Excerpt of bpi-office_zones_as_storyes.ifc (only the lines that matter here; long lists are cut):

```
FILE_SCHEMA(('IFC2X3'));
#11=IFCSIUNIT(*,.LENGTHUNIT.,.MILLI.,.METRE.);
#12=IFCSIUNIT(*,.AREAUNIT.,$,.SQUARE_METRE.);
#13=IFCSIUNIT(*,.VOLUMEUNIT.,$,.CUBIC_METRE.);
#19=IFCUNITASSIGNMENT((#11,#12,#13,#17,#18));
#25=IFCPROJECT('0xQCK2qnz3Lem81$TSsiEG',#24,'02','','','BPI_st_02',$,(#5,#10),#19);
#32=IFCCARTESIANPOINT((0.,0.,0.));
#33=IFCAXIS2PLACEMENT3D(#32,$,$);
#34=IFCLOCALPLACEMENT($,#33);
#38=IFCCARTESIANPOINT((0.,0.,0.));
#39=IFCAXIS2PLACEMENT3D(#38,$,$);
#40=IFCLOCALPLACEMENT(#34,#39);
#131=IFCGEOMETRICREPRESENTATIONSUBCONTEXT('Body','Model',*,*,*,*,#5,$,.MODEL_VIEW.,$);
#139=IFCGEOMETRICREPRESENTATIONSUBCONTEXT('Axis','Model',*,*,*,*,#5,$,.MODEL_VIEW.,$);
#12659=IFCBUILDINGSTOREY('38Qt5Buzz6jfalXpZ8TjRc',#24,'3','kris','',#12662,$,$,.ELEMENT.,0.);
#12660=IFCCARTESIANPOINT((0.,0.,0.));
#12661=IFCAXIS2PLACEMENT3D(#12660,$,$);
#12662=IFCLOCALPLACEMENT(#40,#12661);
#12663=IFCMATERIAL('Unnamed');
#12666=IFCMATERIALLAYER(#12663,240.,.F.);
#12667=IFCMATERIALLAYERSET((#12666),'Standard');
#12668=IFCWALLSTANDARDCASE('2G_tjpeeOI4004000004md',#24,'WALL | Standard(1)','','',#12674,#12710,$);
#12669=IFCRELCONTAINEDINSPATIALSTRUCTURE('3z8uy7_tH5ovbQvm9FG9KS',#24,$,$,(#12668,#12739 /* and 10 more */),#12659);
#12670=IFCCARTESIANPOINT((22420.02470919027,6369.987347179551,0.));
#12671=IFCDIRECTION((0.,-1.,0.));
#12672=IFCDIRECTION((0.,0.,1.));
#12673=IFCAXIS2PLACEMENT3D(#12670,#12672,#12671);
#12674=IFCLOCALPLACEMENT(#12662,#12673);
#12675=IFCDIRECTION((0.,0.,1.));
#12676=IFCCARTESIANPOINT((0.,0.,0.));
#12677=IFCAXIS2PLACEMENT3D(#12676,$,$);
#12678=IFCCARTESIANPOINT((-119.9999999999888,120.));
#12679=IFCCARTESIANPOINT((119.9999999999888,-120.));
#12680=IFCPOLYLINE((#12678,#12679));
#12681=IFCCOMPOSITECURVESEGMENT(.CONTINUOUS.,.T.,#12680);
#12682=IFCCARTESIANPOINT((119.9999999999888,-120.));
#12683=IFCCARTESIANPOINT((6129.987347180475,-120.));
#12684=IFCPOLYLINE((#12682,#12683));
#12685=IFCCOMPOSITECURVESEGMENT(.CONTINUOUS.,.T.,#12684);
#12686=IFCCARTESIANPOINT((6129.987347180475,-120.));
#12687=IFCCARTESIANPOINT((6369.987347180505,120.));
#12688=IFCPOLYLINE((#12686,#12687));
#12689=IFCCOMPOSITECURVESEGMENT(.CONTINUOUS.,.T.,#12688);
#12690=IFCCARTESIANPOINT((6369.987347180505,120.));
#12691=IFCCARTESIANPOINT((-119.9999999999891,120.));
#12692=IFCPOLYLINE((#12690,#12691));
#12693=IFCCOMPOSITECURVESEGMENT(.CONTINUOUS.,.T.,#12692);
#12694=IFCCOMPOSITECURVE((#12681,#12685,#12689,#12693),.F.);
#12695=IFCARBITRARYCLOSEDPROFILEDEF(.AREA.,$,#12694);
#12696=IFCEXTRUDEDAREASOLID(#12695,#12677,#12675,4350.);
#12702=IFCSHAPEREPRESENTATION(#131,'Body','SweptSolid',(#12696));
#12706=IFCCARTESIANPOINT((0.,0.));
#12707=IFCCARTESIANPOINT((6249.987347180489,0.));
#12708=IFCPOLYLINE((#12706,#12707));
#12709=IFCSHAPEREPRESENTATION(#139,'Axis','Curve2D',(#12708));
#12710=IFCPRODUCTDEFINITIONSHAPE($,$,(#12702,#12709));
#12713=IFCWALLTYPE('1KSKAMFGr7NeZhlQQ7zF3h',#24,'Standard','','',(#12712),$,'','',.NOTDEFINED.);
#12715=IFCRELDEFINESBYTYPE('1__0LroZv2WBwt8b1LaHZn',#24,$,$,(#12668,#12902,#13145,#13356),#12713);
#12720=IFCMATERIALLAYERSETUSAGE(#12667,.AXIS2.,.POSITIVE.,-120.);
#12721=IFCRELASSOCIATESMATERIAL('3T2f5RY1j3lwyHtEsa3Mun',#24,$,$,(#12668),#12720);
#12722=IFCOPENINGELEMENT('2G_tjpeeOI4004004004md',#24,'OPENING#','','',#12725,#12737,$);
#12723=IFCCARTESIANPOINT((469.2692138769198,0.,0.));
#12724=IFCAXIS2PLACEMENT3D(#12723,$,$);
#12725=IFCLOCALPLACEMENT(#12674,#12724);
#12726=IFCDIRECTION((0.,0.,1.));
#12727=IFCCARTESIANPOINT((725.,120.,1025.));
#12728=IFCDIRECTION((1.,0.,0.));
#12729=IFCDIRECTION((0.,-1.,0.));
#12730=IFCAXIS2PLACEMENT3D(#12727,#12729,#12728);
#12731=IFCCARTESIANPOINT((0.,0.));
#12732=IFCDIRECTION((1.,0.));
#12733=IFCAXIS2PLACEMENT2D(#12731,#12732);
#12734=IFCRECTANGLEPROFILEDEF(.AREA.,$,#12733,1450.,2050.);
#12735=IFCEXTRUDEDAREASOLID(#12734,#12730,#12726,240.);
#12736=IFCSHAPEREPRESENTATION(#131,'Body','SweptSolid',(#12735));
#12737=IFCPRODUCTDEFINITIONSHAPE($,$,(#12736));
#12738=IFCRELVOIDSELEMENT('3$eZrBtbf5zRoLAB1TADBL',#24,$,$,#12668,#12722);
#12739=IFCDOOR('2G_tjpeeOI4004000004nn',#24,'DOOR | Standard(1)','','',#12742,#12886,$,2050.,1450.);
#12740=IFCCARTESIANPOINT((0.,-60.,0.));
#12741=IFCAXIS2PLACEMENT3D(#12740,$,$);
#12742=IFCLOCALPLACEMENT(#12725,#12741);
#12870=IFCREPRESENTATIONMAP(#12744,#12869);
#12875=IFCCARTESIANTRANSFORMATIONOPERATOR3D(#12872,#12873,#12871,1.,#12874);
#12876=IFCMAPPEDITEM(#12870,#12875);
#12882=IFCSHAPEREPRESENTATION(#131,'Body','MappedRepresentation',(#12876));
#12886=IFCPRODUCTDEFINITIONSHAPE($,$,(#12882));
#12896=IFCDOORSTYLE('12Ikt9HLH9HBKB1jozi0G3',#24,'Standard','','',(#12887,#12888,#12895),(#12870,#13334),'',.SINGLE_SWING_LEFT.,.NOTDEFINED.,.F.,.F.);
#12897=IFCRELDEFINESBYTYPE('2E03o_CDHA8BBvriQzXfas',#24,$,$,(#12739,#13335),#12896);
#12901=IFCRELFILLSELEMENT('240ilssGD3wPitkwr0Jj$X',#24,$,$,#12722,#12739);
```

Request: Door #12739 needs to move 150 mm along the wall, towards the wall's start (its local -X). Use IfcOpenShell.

```python
import ifcopenshell
import ifcopenshell.api.geometry
import ifcopenshell.util.placement
import ifcopenshell.util.unit

model = ifcopenshell.open("bpi-office_zones_as_storyes.ifc")
unit_scale = ifcopenshell.util.unit.calculate_unit_scale(model)

door = model.by_id(12739)
opening = door.FillsVoids[0].RelatingOpeningElement
wall = opening.VoidsElements[0].RelatingBuildingElement

wall_matrix = ifcopenshell.util.placement.get_local_placement(wall.ObjectPlacement)
shift = wall_matrix[:3, 0] * -0.15 / unit_scale
before = ifcopenshell.util.placement.get_local_placement(door.ObjectPlacement)[:3, 3].copy()

# The door is placed relative to its opening, so it follows when the opening moves.
matrix = ifcopenshell.util.placement.get_local_placement(opening.ObjectPlacement)
matrix[:3, 3] += shift
ifcopenshell.api.geometry.edit_object_placement(
    model, product=opening, matrix=matrix, is_si=False, should_transform_children=True
)

after = ifcopenshell.util.placement.get_local_placement(door.ObjectPlacement)[:3, 3]
print("door moved by", (after - before).round(3) + 0.0)

model.write("bpi-office_zones_as_storyes_v2.ifc")
```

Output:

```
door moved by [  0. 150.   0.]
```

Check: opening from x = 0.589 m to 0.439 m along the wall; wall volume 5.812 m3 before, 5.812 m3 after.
